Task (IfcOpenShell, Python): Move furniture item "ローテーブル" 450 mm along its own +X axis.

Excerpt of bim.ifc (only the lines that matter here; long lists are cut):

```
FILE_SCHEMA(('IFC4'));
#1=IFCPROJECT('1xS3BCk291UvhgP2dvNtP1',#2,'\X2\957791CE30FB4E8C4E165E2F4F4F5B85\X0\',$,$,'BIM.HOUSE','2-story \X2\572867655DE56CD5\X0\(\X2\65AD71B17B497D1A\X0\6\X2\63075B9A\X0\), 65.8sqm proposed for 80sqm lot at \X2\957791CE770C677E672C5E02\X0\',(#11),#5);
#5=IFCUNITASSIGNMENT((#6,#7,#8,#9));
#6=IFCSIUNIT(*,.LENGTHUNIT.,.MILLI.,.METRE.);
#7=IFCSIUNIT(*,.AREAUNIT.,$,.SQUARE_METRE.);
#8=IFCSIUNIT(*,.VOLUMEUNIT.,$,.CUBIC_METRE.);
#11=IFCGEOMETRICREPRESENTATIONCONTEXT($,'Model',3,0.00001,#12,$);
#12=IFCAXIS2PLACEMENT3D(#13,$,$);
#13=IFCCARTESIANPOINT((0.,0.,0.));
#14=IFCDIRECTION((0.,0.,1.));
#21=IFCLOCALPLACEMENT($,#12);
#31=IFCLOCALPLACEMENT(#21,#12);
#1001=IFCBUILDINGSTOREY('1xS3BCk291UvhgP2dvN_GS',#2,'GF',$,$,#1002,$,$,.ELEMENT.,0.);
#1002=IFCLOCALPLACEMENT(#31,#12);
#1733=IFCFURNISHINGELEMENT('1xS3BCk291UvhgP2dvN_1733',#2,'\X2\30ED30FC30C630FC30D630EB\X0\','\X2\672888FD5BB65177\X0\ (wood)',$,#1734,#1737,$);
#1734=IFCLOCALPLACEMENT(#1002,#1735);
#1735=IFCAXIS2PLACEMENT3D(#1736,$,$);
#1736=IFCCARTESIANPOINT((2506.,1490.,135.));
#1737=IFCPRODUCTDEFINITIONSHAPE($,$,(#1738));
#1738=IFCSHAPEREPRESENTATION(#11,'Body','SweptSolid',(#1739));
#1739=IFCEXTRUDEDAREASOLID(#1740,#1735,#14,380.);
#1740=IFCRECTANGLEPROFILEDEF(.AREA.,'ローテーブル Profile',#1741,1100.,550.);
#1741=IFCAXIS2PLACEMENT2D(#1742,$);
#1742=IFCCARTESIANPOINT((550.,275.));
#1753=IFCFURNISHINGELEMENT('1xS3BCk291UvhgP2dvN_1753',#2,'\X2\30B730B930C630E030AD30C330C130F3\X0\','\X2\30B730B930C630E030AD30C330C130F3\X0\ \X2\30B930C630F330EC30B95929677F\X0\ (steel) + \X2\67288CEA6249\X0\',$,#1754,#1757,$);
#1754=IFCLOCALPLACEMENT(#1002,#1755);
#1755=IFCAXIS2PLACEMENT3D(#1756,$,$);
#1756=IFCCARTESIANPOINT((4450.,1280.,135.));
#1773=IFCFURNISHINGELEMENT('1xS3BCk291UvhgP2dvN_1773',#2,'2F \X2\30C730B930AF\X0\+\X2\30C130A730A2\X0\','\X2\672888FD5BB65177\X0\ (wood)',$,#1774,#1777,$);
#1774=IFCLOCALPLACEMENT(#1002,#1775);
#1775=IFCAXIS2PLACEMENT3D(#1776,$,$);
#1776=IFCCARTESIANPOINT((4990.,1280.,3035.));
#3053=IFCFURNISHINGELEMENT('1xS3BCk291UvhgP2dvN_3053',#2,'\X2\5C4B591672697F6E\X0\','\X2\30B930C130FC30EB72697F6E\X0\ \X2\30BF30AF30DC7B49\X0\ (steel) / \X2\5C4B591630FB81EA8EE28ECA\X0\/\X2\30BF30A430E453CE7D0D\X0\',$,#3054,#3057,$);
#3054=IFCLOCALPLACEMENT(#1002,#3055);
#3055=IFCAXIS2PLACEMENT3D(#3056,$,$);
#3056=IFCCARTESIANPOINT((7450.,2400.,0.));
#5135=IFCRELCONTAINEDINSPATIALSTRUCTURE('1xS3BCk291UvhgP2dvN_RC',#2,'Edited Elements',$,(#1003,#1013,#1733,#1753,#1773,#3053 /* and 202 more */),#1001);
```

```python
import ifcopenshell
import ifcopenshell.api.geometry
import ifcopenshell.util.placement

model = ifcopenshell.open("bim.ifc")

item = model.by_guid("1xS3BCk291UvhgP2dvN_1733")
matrix = ifcopenshell.util.placement.get_local_placement(item.ObjectPlacement)
matrix[:3, 3] += matrix[:3, 0] * 450.0
ifcopenshell.api.geometry.edit_object_placement(model, product=item, matrix=matrix, is_si=False)

print(ifcopenshell.util.placement.get_local_placement(item.ObjectPlacement).round(3) + 0.0)

model.write("bim_rev.ifc")
```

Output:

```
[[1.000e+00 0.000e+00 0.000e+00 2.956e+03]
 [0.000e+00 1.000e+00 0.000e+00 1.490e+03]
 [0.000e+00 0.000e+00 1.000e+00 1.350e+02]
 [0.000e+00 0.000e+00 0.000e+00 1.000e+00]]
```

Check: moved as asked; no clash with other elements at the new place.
